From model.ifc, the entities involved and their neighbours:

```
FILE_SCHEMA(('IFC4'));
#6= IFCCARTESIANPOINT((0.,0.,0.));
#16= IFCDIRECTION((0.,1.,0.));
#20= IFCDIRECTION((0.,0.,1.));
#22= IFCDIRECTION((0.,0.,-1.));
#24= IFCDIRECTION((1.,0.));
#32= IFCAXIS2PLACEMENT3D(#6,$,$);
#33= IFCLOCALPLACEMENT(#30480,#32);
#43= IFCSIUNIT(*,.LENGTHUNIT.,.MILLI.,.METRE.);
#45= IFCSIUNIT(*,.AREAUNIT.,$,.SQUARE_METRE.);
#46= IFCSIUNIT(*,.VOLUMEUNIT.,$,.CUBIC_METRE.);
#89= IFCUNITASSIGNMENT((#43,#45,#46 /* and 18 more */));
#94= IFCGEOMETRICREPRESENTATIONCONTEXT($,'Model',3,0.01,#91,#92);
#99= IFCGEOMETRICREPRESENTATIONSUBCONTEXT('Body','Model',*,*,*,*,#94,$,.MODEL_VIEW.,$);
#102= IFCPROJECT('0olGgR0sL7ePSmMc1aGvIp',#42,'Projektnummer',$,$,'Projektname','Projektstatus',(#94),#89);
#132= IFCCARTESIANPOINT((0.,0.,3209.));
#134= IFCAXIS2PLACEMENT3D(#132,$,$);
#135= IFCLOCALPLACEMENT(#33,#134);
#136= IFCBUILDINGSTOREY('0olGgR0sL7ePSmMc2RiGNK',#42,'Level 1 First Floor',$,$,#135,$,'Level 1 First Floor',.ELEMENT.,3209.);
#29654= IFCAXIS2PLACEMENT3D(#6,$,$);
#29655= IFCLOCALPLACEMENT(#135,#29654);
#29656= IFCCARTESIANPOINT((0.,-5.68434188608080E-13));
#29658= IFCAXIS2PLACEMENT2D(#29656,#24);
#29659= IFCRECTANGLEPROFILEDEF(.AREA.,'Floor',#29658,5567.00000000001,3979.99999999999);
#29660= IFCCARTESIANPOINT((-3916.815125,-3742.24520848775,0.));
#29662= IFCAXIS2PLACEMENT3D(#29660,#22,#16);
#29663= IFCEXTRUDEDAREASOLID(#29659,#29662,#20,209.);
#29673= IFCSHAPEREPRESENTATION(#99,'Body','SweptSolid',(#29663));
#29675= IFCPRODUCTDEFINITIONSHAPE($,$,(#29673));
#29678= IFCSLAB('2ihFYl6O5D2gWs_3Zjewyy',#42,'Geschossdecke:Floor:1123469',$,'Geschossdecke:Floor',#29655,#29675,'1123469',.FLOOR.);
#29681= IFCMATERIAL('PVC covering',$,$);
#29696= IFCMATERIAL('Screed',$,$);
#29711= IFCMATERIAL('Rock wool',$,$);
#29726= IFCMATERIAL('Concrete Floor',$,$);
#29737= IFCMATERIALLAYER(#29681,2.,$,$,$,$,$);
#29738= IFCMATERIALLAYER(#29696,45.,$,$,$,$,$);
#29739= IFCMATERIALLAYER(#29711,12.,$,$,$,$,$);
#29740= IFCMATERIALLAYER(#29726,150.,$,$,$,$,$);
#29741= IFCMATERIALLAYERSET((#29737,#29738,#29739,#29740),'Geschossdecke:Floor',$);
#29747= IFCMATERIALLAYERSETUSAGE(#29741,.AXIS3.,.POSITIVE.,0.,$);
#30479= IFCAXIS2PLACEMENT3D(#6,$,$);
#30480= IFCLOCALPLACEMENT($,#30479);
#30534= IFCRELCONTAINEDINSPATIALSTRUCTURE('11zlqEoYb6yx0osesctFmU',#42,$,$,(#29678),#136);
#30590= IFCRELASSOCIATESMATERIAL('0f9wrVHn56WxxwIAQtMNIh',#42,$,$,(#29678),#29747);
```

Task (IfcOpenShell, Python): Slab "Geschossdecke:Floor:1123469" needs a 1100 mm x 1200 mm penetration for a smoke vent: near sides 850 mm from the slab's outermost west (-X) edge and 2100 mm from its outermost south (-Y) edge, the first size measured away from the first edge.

```python
import numpy as np
import ifcopenshell
import ifcopenshell.api.feature
import ifcopenshell.api.geometry
import ifcopenshell.api.root
import ifcopenshell.geom
import ifcopenshell.util.placement
import ifcopenshell.util.representation
import ifcopenshell.util.shape
import ifcopenshell.util.unit

model = ifcopenshell.open("model.ifc")
unit_scale = ifcopenshell.util.unit.calculate_unit_scale(model)
settings = ifcopenshell.geom.settings()


def volume(element):
    """Net volume in cubic metres, openings subtracted."""
    shape = ifcopenshell.geom.create_shape(settings, element)
    return ifcopenshell.util.shape.get_volume(shape.geometry)


slab = model.by_guid("2ihFYl6O5D2gWs_3Zjewyy")
before = volume(slab)

# Extent in the slab's own axes, in metres. The edges named are its -X and -Y sides.
slab_shape = ifcopenshell.geom.create_shape(settings, slab)
vertices = ifcopenshell.util.shape.get_vertices(slab_shape.geometry)
x_min, y_min, bottom = vertices.min(axis=0)
top = vertices[:, 2].max()

opening = ifcopenshell.api.root.create_entity(model, ifc_class="IfcOpeningElement", name="Smoke vent opening", predefined_type="OPENING")
context = ifcopenshell.util.representation.get_context(model, "Model", "Body", "MODEL_VIEW")
width, depth = 1.1, 1.2
outline = [(0.0, 0.0), (width, 0.0), (width, depth), (0.0, depth), (0.0, 0.0)]
# Overshoot both faces by 50 mm so the cut is clean.
shape = ifcopenshell.api.geometry.add_slab_representation(
    model, context=context, depth=top - bottom + 0.1, polyline=outline
)
ifcopenshell.api.geometry.assign_representation(model, product=opening, representation=shape)

matrix = ifcopenshell.util.placement.get_local_placement(slab.ObjectPlacement)
matrix[:, 3] = matrix @ np.append(np.array([x_min + 0.85, y_min + 2.1, bottom - 0.05]) / unit_scale, 1.0)
ifcopenshell.api.geometry.edit_object_placement(model, product=opening, matrix=matrix, is_si=False)
ifcopenshell.api.feature.add_feature(model, feature=opening, element=slab)

after = volume(slab)

print(f"slab volume {before:.3f} -> {after:.3f} m3")

model.write("model_edited.ifc")
```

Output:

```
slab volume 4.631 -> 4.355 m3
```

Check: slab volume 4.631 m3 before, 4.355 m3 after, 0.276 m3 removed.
